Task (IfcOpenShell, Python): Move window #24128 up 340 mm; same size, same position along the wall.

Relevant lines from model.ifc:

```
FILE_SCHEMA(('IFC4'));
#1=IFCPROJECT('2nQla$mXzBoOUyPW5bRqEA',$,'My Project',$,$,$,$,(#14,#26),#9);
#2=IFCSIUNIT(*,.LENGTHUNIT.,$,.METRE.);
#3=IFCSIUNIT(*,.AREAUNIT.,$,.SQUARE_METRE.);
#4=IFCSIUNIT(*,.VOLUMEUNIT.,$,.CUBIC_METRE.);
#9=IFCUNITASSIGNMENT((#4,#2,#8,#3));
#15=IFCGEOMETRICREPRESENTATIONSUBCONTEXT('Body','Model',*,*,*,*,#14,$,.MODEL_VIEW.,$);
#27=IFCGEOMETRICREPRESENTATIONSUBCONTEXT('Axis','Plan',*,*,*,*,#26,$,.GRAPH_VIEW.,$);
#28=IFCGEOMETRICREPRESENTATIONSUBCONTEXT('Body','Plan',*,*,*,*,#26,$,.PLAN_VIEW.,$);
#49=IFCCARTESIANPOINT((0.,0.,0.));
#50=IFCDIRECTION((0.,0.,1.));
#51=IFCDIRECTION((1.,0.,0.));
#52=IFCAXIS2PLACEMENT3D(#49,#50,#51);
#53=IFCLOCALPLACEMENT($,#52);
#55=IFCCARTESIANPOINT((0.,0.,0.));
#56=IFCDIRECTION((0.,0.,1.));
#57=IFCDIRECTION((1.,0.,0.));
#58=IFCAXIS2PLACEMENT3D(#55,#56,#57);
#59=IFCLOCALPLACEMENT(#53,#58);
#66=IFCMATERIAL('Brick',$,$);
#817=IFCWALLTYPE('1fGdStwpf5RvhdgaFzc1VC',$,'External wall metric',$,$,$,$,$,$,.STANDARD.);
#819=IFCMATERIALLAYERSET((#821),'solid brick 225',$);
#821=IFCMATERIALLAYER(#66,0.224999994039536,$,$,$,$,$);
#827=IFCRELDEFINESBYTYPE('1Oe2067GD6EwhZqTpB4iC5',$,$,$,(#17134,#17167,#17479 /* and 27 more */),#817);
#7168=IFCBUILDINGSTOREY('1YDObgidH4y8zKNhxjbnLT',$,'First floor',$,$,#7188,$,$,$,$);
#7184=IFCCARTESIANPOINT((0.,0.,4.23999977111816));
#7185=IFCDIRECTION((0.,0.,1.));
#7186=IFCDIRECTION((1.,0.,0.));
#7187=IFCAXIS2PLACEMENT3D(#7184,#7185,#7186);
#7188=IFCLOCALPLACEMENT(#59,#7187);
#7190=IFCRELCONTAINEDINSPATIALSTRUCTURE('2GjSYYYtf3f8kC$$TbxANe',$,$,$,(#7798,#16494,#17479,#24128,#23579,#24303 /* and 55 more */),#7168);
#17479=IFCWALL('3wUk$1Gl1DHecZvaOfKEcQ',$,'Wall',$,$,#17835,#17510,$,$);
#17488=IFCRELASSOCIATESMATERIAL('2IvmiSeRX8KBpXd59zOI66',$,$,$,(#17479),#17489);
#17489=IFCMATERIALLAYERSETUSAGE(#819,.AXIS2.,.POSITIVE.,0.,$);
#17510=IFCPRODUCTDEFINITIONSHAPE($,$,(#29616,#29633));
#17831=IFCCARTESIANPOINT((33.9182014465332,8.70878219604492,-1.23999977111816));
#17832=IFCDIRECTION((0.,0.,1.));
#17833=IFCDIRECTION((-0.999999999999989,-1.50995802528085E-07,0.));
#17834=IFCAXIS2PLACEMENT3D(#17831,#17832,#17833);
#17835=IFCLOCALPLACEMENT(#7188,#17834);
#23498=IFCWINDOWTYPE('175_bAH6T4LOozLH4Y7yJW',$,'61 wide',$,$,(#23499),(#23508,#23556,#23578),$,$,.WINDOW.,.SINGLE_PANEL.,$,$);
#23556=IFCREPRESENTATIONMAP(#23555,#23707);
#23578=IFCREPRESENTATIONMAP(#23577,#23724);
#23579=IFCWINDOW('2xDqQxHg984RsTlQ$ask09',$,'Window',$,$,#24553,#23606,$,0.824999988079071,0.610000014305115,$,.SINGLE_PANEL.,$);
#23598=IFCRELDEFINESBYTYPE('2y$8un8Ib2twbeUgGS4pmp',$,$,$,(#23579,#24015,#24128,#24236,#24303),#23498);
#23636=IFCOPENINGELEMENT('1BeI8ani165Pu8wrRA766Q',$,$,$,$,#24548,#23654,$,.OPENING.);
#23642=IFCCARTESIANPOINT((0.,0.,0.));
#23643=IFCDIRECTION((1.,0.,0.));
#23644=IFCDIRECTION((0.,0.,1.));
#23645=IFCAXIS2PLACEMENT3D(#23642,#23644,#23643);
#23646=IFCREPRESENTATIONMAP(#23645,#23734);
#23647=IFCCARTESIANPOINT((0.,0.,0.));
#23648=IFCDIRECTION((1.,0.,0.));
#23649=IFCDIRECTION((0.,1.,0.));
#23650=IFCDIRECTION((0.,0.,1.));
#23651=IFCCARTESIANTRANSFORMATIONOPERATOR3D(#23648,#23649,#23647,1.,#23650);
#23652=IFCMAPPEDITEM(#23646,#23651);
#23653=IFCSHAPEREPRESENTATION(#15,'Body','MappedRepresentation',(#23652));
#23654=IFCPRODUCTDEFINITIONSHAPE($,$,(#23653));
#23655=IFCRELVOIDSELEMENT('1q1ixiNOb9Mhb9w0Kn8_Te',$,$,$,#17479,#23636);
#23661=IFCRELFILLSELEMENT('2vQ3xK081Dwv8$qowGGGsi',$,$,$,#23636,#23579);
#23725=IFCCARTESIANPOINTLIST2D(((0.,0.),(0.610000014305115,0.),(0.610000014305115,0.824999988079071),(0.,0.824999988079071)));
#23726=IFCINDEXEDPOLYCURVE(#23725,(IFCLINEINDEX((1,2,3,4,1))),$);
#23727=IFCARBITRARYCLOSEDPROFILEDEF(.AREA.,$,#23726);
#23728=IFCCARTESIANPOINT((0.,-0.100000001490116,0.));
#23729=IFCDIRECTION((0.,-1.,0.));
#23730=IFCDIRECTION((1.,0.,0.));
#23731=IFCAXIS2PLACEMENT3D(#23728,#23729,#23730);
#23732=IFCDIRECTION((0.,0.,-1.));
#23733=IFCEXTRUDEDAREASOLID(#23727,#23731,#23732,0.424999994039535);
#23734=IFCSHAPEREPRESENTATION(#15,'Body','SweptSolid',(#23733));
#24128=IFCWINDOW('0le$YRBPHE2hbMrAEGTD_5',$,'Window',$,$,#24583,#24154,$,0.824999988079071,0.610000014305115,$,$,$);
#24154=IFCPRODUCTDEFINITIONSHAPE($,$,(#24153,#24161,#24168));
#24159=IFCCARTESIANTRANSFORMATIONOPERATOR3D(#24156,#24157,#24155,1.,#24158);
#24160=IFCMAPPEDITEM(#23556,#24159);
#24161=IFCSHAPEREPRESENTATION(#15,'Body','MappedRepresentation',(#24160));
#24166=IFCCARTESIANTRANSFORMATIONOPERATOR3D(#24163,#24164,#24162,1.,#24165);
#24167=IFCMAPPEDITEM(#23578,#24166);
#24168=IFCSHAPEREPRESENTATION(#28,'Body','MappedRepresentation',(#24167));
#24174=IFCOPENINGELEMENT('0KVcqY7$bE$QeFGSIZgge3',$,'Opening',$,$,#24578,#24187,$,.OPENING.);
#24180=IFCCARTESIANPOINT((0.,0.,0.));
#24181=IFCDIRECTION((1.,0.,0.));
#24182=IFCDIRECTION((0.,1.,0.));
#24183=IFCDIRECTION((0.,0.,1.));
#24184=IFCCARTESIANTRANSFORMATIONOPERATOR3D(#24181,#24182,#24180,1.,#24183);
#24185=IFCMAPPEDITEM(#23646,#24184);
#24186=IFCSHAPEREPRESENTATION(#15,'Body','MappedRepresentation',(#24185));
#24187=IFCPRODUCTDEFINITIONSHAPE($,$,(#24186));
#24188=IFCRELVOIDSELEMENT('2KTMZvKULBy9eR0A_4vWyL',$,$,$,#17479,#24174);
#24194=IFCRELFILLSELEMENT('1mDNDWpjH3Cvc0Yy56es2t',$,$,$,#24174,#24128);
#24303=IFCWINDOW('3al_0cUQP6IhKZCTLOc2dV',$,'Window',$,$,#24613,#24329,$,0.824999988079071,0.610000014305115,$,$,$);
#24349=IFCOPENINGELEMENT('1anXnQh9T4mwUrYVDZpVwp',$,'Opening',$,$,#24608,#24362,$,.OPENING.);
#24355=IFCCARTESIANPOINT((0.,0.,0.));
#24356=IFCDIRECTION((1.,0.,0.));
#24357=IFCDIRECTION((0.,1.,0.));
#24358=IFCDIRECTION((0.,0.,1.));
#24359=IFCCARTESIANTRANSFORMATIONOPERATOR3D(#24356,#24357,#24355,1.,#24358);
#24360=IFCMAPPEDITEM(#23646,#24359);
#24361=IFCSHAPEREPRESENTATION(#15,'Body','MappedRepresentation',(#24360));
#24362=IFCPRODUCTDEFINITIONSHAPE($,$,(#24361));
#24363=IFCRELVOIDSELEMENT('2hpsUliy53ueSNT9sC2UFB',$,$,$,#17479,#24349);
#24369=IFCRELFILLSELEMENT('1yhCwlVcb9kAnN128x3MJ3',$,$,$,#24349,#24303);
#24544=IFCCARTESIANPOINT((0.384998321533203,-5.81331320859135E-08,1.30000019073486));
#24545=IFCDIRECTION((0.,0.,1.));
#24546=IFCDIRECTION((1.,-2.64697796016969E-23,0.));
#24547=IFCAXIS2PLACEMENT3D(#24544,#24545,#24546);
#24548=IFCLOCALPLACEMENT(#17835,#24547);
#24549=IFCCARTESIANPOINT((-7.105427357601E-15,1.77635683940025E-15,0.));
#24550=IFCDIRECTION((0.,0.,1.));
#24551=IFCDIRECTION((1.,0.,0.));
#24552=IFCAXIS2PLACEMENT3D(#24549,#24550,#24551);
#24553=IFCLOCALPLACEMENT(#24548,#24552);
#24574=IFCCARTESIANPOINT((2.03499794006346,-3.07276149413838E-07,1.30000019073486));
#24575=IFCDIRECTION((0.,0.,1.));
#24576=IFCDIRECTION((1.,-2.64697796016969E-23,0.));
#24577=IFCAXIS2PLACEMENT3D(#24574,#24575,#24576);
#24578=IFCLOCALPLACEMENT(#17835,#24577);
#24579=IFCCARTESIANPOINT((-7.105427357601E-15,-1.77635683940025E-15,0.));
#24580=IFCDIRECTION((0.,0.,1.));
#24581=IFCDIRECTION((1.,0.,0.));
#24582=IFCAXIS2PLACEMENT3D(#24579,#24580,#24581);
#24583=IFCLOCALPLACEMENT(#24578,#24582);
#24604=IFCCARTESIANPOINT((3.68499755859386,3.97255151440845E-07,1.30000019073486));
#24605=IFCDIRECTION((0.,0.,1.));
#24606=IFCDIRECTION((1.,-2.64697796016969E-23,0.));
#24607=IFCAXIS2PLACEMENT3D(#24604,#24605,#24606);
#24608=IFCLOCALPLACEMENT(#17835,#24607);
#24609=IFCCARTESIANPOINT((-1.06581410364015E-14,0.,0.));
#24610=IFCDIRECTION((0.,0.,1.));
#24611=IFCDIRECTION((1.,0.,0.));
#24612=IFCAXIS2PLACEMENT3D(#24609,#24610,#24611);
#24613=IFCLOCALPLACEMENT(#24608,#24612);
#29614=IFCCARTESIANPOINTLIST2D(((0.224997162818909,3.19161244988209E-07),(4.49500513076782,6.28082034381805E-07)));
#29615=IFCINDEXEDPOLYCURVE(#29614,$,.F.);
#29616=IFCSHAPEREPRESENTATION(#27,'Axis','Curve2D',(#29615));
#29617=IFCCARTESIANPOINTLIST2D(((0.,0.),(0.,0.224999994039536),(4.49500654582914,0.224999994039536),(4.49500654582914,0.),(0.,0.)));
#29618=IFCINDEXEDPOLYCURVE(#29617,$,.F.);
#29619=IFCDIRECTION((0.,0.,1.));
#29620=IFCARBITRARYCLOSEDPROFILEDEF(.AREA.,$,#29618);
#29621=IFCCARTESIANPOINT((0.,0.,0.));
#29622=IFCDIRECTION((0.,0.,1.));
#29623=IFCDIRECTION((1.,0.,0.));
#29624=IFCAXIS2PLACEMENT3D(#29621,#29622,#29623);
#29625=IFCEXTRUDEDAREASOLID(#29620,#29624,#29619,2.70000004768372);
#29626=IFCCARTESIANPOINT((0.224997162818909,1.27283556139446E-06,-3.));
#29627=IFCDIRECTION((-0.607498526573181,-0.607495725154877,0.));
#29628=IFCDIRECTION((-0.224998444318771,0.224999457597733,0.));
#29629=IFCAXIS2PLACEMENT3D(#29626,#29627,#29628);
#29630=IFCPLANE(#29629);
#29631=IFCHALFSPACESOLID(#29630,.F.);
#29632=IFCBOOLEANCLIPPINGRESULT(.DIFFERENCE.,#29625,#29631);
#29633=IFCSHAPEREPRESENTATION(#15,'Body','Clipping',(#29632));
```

```python
import numpy as np
import ifcopenshell
import ifcopenshell.api.geometry
import ifcopenshell.util.placement
import ifcopenshell.util.unit

model = ifcopenshell.open("model.ifc")
unit_scale = ifcopenshell.util.unit.calculate_unit_scale(model)

window = model.by_id(24128)
opening = window.FillsVoids[0].RelatingOpeningElement
dz = 0.34 / unit_scale

shift = np.array([0.0, 0.0, dz])
# The window is placed relative to its opening, so it follows when the opening moves.
matrix = ifcopenshell.util.placement.get_local_placement(opening.ObjectPlacement)
matrix[:3, 3] += shift
ifcopenshell.api.geometry.edit_object_placement(
    model, product=opening, matrix=matrix, is_si=False, should_transform_children=True
)

print(f"moved by {dz * unit_scale:+.3f} m")

model.write("model_edited.ifc")
```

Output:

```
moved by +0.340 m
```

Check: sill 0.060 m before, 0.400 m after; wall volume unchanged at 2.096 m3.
